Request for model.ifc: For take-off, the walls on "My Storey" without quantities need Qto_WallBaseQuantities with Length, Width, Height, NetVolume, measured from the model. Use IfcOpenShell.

First a look at what the model holds.

```python
import ifcopenshell
import ifcopenshell.util.element
import ifcopenshell.util.unit

model = ifcopenshell.open("model.ifc")
print(model.schema)
for unit_type in ("LENGTHUNIT", "AREAUNIT", "VOLUMEUNIT"):
    print(unit_type, ifcopenshell.util.unit.calculate_unit_scale(model, unit_type))
storey = next(s for s in model.by_type("IfcBuildingStorey") if s.Name == "My Storey")
walls = [e for e in ifcopenshell.util.element.get_decomposition(storey) if e.is_a("IfcWall")]
for e in sorted(walls, key=lambda e: e.id()):
    print(e.id(), e.is_a(), e.Name, list(ifcopenshell.util.element.get_psets(e, qtos_only=True)), sep=" | ")
```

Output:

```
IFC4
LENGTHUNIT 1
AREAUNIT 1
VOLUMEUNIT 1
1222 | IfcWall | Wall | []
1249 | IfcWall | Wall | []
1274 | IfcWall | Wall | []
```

```python
import ifcopenshell
import ifcopenshell.api.pset
import ifcopenshell.geom
import ifcopenshell.util.element
import ifcopenshell.util.shape
import ifcopenshell.util.unit

model = ifcopenshell.open("model.ifc")
unit_scale = ifcopenshell.util.unit.calculate_unit_scale(model)
volume_scale = ifcopenshell.util.unit.calculate_unit_scale(model, "VOLUMEUNIT")
settings = ifcopenshell.geom.settings()

storey = next(s for s in model.by_type("IfcBuildingStorey") if s.Name == "My Storey")
walls = [e for e in ifcopenshell.util.element.get_decomposition(storey) if e.is_a("IfcWall")]

for e in sorted(walls, key=lambda e: e.id()):
    if ifcopenshell.util.element.get_psets(e, qtos_only=True, should_inherit=False):
        continue
    # Geometry comes back in metres, in the element's own axes.
    shape = ifcopenshell.geom.create_shape(settings, e)
    values = {
        "Length": ifcopenshell.util.shape.get_x(shape.geometry) / unit_scale,
        "Width": ifcopenshell.util.shape.get_y(shape.geometry) / unit_scale,
        "Height": ifcopenshell.util.shape.get_z(shape.geometry) / unit_scale,
        "NetVolume": ifcopenshell.util.shape.get_volume(shape.geometry) / volume_scale,
    }
    qto = ifcopenshell.api.pset.add_qto(model, product=e, name="Qto_WallBaseQuantities")
    ifcopenshell.api.pset.edit_qto(model, qto=qto, properties=values)
    print(e.id(), {k: round(v, 3) for k, v in values.items()})

model.write("model_updated.ifc")
```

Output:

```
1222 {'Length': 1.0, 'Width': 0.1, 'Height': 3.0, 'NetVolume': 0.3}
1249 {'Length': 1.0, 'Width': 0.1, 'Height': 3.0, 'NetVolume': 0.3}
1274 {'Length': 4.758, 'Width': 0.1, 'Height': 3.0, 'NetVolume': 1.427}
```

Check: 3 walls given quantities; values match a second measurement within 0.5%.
